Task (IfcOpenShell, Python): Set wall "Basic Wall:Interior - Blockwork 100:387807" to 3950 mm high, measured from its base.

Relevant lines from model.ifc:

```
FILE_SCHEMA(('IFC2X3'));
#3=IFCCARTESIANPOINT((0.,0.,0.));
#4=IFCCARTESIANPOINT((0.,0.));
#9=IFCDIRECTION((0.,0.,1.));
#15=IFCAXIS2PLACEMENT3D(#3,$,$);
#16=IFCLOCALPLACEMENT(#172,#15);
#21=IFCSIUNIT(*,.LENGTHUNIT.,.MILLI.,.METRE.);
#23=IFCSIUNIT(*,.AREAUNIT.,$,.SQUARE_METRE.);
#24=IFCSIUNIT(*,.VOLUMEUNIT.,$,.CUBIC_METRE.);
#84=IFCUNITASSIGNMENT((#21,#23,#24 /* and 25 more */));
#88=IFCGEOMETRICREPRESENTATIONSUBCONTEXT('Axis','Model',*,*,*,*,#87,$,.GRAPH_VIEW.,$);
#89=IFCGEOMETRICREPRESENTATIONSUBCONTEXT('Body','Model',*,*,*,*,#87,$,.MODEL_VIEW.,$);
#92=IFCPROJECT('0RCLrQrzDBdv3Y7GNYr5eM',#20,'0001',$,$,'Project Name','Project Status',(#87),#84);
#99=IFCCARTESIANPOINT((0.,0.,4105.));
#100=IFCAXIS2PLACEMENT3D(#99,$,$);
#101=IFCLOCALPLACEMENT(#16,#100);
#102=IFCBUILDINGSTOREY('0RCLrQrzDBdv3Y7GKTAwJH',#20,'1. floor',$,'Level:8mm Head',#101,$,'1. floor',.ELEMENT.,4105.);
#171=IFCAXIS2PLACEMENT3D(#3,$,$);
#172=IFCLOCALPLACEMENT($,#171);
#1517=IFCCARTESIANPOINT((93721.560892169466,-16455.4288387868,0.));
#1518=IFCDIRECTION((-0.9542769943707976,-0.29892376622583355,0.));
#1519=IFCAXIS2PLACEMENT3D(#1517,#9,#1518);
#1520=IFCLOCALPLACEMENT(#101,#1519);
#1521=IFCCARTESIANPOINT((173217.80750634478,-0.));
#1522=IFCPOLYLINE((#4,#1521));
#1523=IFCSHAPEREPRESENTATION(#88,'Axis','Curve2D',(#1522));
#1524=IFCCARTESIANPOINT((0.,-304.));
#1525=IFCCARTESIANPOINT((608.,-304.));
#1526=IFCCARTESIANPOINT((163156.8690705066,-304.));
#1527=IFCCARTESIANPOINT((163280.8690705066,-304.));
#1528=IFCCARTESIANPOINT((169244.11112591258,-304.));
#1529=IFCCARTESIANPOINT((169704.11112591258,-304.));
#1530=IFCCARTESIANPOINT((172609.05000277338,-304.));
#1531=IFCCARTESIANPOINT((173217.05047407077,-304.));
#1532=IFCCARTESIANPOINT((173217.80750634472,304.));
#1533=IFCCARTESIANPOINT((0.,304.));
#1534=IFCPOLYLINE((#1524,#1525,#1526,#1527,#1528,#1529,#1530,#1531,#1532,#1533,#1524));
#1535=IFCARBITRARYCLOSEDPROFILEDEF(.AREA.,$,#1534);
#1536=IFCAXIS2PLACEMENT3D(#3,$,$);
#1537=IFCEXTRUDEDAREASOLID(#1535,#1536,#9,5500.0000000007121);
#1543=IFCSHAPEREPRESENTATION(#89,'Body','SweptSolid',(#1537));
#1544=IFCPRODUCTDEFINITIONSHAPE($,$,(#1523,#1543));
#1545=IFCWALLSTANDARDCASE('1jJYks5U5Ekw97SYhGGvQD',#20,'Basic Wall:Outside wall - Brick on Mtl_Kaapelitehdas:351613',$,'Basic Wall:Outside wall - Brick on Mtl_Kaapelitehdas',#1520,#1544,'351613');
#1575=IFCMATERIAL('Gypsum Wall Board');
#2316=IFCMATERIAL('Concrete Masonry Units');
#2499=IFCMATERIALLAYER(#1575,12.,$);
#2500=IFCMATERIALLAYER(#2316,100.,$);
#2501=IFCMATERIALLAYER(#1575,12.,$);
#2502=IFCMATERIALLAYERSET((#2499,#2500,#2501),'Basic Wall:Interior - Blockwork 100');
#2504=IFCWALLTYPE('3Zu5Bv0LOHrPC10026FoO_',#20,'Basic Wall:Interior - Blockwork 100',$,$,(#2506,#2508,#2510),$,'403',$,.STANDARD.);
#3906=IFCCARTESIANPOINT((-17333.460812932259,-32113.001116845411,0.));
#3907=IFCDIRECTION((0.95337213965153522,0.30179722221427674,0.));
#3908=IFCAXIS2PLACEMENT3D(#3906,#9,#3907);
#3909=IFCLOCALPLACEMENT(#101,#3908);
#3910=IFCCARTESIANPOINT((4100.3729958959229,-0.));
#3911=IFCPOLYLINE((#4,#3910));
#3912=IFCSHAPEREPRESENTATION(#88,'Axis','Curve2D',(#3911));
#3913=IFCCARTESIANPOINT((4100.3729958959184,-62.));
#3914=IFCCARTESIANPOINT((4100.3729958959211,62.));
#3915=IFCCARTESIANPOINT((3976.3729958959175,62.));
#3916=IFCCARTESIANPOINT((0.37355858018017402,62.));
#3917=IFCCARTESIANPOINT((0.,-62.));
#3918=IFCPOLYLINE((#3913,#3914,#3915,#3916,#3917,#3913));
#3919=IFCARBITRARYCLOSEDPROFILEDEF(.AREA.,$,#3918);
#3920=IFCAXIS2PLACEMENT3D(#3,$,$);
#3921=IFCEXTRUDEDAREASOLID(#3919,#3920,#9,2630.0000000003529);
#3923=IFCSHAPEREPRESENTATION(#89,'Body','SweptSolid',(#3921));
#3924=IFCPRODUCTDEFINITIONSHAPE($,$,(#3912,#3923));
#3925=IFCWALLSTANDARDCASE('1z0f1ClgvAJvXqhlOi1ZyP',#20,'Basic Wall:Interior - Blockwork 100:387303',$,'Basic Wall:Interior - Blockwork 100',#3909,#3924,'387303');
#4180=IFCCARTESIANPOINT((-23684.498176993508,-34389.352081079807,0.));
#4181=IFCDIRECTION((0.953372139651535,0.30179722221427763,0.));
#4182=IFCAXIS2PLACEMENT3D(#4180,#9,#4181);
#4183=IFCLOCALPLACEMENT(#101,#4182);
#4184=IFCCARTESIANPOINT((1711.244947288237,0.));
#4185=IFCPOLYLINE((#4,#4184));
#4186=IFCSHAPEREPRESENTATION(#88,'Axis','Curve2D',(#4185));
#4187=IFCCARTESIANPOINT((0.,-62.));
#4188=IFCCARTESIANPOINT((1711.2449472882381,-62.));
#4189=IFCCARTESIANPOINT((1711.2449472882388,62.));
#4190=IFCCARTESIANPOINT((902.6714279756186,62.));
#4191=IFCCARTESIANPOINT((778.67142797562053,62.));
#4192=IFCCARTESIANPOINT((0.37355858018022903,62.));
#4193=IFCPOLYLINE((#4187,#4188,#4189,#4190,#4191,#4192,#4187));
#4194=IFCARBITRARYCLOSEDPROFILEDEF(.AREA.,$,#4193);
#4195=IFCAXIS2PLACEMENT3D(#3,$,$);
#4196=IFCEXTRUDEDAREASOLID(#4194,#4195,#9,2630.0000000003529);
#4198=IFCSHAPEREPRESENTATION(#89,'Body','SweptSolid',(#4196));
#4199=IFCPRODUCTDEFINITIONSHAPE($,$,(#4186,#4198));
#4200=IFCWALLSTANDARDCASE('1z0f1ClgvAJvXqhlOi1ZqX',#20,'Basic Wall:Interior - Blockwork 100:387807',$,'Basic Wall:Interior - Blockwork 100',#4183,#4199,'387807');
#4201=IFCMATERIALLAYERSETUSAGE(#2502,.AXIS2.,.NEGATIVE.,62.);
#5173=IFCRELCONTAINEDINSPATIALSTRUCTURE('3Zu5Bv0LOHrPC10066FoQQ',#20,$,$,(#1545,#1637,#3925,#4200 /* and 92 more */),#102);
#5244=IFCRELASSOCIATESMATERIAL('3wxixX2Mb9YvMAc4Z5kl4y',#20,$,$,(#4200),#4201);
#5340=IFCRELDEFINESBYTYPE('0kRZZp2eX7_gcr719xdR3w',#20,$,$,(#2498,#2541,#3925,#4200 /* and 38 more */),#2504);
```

```python
import ifcopenshell
import ifcopenshell.geom
import ifcopenshell.util.representation
import ifcopenshell.util.shape

model = ifcopenshell.open("model.ifc")
settings = ifcopenshell.geom.settings()


def volume(element):
    """Net volume in cubic metres, openings subtracted."""
    shape = ifcopenshell.geom.create_shape(settings, element)
    return ifcopenshell.util.shape.get_volume(shape.geometry)


wall = model.by_guid("1z0f1ClgvAJvXqhlOi1ZqX")
before = volume(wall)

body = ifcopenshell.util.representation.get_representation(wall, "Model", "Body")
solid = body.Items[0]
old_height = solid.Depth
solid.Depth = 3950.0
after = volume(wall)

print(f"height {old_height:g} -> {solid.Depth:g}, volume {before:.3f} -> {after:.3f} m3")

model.write("model_rev.ifc")
```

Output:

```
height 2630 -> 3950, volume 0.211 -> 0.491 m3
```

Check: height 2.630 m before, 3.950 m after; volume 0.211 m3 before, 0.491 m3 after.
